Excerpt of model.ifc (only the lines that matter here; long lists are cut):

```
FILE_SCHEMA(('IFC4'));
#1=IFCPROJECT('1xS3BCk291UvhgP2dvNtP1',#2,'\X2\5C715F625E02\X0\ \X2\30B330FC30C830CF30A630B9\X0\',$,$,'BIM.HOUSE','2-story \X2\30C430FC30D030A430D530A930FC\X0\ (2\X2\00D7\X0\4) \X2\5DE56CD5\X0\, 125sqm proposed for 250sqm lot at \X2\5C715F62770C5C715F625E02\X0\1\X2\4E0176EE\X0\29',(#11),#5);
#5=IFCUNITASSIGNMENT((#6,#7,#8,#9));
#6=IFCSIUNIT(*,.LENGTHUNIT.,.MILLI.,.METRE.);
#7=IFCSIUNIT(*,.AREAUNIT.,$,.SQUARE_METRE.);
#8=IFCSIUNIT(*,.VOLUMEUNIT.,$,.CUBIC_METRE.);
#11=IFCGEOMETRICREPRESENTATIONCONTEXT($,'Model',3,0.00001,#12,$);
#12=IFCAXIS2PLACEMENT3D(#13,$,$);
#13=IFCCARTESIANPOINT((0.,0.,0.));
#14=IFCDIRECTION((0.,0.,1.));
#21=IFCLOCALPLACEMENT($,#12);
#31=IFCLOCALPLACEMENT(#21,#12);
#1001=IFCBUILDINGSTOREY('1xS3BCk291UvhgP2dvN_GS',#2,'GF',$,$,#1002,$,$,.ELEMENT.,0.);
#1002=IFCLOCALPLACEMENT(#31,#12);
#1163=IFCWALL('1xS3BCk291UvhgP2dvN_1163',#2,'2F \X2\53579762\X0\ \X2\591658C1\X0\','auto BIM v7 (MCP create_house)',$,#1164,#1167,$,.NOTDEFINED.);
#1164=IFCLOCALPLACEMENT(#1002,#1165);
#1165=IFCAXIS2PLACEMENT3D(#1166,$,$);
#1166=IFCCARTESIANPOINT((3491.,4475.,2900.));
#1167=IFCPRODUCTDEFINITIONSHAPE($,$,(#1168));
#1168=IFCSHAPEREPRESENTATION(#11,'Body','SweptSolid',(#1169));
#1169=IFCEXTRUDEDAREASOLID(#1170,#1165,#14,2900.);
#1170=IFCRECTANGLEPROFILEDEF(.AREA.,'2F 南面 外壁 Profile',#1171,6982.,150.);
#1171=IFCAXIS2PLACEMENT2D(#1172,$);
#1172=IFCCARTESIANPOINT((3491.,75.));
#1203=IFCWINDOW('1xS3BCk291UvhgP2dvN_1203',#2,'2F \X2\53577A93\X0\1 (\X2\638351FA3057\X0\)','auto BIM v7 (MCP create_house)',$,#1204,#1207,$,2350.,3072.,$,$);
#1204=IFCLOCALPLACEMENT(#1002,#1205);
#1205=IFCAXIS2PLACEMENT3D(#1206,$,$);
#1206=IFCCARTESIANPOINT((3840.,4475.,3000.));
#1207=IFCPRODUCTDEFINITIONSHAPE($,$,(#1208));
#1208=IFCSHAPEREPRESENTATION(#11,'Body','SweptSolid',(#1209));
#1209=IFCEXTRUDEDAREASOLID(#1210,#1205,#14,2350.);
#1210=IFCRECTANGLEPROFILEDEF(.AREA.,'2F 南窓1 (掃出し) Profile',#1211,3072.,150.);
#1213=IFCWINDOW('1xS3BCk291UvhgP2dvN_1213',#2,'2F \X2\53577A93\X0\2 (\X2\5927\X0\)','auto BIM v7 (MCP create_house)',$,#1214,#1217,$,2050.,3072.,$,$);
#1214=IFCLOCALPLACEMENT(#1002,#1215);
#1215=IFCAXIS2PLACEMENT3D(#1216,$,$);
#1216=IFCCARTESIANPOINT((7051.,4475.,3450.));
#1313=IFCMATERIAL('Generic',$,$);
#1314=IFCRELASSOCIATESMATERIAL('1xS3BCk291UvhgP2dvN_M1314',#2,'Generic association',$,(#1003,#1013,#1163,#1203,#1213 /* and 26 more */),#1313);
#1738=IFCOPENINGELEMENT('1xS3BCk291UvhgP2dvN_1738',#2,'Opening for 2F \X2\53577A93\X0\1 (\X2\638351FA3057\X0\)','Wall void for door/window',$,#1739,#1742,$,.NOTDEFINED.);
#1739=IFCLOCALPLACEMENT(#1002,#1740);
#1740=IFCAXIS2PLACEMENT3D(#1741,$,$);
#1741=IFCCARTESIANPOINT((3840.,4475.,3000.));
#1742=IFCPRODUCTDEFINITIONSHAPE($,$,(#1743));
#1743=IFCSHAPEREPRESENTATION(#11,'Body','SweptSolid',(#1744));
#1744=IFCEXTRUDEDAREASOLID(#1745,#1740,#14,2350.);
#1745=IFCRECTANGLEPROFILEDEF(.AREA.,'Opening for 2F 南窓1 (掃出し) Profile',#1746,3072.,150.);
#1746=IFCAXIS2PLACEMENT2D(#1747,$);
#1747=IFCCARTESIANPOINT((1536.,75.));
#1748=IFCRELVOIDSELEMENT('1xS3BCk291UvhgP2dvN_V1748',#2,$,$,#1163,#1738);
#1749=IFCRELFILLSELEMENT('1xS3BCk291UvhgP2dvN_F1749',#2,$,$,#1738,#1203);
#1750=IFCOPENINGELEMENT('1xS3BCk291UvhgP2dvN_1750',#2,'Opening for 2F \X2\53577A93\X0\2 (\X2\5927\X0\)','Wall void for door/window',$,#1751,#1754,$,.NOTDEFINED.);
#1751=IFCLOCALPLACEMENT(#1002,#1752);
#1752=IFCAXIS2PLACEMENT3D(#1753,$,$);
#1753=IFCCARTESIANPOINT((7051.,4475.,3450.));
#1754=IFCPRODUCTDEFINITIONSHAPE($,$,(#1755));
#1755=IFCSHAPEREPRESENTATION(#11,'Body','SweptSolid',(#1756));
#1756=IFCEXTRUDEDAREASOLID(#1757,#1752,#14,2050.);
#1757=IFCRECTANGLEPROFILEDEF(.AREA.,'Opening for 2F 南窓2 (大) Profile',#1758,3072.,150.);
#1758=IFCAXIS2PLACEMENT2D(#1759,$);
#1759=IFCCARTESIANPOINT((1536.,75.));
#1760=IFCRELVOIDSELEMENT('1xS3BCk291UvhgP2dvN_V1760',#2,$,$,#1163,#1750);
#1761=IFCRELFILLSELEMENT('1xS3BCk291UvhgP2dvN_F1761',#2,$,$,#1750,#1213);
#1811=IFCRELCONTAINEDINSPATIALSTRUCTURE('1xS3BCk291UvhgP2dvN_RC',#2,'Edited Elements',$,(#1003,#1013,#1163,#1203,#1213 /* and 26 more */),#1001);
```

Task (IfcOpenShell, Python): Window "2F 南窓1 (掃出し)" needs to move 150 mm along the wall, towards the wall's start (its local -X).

```python
import ifcopenshell
import ifcopenshell.api.geometry
import ifcopenshell.util.placement

model = ifcopenshell.open("model.ifc")

window = model.by_id(1203)
opening = window.FillsVoids[0].RelatingOpeningElement
wall = opening.VoidsElements[0].RelatingBuildingElement

wall_matrix = ifcopenshell.util.placement.get_local_placement(wall.ObjectPlacement)
shift = wall_matrix[:3, 0] * -150.0
before = ifcopenshell.util.placement.get_local_placement(window.ObjectPlacement)[:3, 3].copy()

# The window is not placed relative to its opening, so move both.
for product in (opening, window):
    matrix = ifcopenshell.util.placement.get_local_placement(product.ObjectPlacement)
    matrix[:3, 3] += shift
    ifcopenshell.api.geometry.edit_object_placement(model, product=product, matrix=matrix, is_si=False)

after = ifcopenshell.util.placement.get_local_placement(window.ObjectPlacement)[:3, 3]
print("window moved by", (after - before).round(3) + 0.0)

model.write("model_edited.ifc")
```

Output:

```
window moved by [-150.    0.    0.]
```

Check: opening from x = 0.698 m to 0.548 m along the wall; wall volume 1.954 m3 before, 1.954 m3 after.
